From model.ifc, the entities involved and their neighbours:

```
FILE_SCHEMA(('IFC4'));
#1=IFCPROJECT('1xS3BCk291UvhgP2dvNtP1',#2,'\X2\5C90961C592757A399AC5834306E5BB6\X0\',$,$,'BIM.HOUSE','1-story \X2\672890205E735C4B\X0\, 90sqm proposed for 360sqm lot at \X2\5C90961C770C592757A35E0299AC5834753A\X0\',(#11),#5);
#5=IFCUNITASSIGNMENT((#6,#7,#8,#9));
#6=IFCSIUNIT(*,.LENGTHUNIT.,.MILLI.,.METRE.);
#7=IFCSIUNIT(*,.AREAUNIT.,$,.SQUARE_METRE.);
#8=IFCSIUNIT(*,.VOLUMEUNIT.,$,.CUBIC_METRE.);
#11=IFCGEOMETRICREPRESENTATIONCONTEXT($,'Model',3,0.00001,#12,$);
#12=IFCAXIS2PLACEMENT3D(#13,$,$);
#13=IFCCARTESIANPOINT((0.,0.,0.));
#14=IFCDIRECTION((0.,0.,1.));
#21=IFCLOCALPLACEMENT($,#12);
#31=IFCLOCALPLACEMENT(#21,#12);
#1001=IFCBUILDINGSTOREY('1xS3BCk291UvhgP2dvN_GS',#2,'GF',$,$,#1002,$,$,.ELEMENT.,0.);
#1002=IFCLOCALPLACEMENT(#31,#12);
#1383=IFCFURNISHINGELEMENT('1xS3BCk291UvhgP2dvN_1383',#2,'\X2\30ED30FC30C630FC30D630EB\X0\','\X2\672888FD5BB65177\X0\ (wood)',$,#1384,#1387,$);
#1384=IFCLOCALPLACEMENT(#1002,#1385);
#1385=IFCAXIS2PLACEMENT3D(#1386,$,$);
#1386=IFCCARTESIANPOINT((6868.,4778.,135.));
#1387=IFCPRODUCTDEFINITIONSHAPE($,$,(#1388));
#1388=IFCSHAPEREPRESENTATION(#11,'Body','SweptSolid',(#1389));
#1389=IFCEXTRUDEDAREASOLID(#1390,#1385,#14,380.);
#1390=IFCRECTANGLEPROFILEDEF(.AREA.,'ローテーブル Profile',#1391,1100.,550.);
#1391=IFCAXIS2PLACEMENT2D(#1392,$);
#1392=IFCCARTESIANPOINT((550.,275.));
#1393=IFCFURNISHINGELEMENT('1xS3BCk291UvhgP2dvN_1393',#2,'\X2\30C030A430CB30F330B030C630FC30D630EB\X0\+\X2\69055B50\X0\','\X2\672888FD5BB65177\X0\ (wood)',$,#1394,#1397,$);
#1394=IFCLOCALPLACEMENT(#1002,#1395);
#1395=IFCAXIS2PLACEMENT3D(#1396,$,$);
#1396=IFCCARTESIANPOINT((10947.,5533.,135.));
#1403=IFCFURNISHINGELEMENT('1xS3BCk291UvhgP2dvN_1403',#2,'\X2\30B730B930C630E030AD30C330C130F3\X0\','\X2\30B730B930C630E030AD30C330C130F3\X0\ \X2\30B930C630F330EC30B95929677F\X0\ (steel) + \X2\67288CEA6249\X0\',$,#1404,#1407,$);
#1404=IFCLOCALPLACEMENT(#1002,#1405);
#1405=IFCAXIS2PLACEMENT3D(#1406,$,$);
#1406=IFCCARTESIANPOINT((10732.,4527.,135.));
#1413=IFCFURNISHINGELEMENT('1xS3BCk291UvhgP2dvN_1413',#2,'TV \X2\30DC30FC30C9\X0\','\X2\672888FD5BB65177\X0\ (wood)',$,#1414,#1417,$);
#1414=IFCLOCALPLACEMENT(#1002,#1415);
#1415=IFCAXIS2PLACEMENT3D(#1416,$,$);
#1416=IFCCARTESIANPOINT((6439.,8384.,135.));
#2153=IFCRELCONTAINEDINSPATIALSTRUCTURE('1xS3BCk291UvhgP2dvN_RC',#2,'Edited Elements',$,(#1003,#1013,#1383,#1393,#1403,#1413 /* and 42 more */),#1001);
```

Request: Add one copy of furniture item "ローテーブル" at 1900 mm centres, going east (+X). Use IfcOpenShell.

```python
import numpy as np
import ifcopenshell
import ifcopenshell.api.geometry
import ifcopenshell.api.root
import ifcopenshell.util.element
import ifcopenshell.util.placement
import ifcopenshell.util.unit

model = ifcopenshell.open("model.ifc")
unit_scale = ifcopenshell.util.unit.calculate_unit_scale(model)


def reuse_history(source, copy):
    """copy_class also copies each property set's owner history, people and application; keep the originals."""
    for rel in copy.IsDefinedBy:
        if rel.is_a("IfcRelDefinesByProperties") and (history := rel.RelatingPropertyDefinition.OwnerHistory):
            rel.RelatingPropertyDefinition.OwnerHistory = source.OwnerHistory
            ifcopenshell.util.element.remove_deep2(model, history)


source = model.by_guid("1xS3BCk291UvhgP2dvN_1383")
base = ifcopenshell.util.placement.get_local_placement(source.ObjectPlacement)
step = np.array([1.0, 0.0, 0.0]) * 1.9 / unit_scale

for i in range(1, 2):
    copy = ifcopenshell.api.root.copy_class(model, product=source)
    copy.Representation = ifcopenshell.util.element.copy_deep(
        model, source.Representation, exclude=["IfcGeometricRepresentationContext", "IfcRepresentationMap"]
    )
    reuse_history(source, copy)
    matrix = base.copy()
    matrix[:3, 3] += i * step
    print("added at", matrix[:3, 3].round(3) + 0.0)
    ifcopenshell.api.geometry.edit_object_placement(model, product=copy, matrix=matrix, is_si=False)

model.write("model_edited.ifc")
```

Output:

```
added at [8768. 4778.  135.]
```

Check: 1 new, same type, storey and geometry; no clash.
